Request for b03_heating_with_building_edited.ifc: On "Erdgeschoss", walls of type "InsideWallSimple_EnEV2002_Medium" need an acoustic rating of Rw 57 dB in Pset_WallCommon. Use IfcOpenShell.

First a look at what the model holds.

```python
import ifcopenshell
import ifcopenshell.util.element

model = ifcopenshell.open("b03_heating_with_building_edited.ifc")
print(model.schema)
storey = next(s for s in model.by_type("IfcBuildingStorey") if s.Name == "Erdgeschoss")
walls = [e for e in ifcopenshell.util.element.get_decomposition(storey) if e.is_a("IfcWall")]
seen = {}
for e in walls:
    element_type = ifcopenshell.util.element.get_type(e)
    key = (element_type.Name if element_type != e and element_type else None, ifcopenshell.util.element.get_pset(e, "Pset_WallCommon", "AcousticRating"))
    seen[key] = seen.get(key, 0) + 1
for (name, value), count in sorted(seen.items(), key=str):
    print(count, "x", name, "|", value)
```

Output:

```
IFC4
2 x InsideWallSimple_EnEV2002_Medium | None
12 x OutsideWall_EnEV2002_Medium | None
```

```python
import ifcopenshell
import ifcopenshell.api.pset
import ifcopenshell.util.element

model = ifcopenshell.open("b03_heating_with_building_edited.ifc")

storey = next(s for s in model.by_type("IfcBuildingStorey") if s.Name == "Erdgeschoss")
walls = [e for e in ifcopenshell.util.element.get_decomposition(storey) if e.is_a("IfcWall")]

count = 0
for e in walls:
    element_type = ifcopenshell.util.element.get_type(e)
    if element_type in (None, e) or element_type.Name != "InsideWallSimple_EnEV2002_Medium":
        continue
    found = ifcopenshell.util.element.get_pset(e, "Pset_WallCommon", should_inherit=False)
    if found:
        pset = model.by_id(found["id"])
        if len(ifcopenshell.util.element.get_elements_by_pset(pset)) > 1:
            pset = ifcopenshell.api.pset.unshare_pset(model, products=[e], pset=pset)[0]
    else:
        pset = ifcopenshell.api.pset.add_pset(model, product=e, name="Pset_WallCommon")
    ifcopenshell.api.pset.edit_pset(model, pset=pset, properties={"AcousticRating": "Rw 57 dB"})
    count += 1

print(count, "walls updated")

model.write("b03_heating_with_building_edited_edited.ifc")
```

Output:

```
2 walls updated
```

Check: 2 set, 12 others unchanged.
